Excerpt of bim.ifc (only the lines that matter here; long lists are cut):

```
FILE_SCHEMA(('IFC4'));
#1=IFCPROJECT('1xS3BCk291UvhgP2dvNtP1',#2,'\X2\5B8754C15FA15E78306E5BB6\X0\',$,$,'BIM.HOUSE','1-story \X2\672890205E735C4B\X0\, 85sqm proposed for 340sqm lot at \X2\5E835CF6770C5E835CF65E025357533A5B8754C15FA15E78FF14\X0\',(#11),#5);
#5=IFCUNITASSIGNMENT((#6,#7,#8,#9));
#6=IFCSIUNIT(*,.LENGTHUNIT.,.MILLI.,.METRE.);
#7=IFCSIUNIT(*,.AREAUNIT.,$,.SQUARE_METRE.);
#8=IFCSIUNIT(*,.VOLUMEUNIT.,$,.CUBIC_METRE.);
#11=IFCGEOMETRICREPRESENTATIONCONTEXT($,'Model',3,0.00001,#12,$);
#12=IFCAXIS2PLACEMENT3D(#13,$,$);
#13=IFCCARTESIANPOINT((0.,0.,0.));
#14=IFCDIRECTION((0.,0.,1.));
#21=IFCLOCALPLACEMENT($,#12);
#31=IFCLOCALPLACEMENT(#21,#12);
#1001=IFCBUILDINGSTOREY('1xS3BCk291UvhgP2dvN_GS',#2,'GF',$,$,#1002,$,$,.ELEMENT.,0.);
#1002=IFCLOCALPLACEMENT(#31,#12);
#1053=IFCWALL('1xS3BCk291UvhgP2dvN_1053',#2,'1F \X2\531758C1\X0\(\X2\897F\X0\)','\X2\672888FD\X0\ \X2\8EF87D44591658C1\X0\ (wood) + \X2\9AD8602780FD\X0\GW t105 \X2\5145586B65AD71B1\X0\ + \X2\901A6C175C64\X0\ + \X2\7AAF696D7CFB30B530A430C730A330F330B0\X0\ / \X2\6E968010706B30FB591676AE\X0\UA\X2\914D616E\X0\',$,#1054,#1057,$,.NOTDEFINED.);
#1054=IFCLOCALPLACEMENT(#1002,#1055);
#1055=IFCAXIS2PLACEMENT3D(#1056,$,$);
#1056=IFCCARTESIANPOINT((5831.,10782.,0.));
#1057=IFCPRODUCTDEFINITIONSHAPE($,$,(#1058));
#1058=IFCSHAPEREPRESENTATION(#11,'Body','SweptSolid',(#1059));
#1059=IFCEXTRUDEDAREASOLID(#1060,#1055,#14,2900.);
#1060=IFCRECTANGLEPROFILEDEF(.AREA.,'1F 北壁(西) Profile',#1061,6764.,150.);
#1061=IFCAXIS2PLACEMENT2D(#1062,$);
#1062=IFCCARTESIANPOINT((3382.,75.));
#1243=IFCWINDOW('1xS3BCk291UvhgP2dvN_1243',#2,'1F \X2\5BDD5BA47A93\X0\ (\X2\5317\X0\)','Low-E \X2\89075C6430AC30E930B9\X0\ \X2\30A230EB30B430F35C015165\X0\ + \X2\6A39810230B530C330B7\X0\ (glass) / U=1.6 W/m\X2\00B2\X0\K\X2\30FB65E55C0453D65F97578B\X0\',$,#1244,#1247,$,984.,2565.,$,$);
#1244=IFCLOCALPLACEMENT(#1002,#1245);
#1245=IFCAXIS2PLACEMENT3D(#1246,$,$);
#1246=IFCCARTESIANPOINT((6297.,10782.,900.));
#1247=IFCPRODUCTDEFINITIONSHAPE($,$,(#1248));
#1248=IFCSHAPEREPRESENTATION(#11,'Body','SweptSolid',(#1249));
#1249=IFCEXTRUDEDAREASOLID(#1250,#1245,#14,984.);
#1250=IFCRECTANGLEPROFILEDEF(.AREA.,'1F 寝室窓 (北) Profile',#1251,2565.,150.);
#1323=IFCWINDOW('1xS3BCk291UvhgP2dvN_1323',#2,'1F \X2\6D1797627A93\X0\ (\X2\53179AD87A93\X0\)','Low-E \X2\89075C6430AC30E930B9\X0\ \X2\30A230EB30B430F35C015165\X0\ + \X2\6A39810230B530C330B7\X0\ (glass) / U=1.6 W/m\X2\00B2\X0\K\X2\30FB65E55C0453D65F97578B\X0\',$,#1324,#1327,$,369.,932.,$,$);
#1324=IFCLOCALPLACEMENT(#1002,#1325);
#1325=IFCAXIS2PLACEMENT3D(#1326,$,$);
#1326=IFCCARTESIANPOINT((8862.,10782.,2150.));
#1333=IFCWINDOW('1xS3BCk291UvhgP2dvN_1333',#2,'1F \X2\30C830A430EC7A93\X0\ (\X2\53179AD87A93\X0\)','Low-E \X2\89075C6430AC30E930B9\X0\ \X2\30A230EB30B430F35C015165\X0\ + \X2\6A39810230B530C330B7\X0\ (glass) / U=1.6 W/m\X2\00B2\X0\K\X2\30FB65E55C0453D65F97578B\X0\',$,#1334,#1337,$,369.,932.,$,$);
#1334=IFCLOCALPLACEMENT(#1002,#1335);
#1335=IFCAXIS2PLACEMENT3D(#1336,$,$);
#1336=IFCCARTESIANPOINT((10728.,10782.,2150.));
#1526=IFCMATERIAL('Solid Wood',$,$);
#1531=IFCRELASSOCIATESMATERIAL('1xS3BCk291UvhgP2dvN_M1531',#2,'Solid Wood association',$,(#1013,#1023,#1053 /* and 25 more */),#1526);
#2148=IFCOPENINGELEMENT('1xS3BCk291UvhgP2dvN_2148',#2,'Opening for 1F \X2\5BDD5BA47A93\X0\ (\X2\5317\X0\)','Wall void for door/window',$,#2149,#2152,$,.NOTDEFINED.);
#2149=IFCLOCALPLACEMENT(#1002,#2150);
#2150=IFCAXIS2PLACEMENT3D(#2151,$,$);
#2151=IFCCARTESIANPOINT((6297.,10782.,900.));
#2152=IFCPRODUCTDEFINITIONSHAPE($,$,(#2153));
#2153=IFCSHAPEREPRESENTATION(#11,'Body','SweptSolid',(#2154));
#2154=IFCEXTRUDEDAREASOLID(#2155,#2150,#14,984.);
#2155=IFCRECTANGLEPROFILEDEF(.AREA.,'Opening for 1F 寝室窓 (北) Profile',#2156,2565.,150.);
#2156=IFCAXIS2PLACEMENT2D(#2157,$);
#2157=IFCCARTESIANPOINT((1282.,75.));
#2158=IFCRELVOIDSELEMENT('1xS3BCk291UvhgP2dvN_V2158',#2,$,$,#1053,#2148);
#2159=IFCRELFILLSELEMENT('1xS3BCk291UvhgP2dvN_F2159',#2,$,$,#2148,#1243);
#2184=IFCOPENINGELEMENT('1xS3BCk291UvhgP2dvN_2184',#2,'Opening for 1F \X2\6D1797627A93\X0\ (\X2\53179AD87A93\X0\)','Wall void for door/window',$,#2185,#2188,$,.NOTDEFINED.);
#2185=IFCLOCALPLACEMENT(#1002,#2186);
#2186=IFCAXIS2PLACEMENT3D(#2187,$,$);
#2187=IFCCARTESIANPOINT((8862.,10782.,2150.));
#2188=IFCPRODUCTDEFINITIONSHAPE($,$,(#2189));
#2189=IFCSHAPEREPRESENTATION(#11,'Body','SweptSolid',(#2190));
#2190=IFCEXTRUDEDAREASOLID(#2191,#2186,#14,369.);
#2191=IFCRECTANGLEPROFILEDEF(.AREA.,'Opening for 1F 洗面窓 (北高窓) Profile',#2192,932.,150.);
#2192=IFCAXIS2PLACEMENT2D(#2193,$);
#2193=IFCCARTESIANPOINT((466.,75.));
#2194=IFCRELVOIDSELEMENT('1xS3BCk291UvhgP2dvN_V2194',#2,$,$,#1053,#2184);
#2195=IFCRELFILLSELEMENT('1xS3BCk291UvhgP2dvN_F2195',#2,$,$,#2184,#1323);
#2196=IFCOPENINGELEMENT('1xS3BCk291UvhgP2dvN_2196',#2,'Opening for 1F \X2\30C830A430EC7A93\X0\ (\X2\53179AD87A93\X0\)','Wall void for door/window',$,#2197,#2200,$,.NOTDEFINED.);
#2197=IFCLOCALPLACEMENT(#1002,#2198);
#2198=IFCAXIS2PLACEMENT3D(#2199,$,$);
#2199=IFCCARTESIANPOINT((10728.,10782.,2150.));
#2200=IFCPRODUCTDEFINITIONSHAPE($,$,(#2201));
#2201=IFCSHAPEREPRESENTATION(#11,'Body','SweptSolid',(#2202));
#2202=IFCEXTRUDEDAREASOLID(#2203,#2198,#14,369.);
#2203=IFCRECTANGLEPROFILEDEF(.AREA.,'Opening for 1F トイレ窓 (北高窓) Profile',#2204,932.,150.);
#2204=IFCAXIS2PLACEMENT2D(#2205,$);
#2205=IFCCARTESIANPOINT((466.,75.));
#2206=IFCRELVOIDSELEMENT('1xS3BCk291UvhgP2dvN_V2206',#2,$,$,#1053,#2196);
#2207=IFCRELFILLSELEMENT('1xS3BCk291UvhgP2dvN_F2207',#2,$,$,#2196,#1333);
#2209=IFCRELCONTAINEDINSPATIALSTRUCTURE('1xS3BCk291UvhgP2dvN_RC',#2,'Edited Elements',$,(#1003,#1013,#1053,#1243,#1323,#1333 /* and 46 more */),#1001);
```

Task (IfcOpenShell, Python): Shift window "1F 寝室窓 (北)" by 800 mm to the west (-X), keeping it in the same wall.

```python
import ifcopenshell
import ifcopenshell.api.geometry
import ifcopenshell.util.placement

model = ifcopenshell.open("bim.ifc")

window = model.by_id(1243)
opening = window.FillsVoids[0].RelatingOpeningElement
wall = opening.VoidsElements[0].RelatingBuildingElement

wall_matrix = ifcopenshell.util.placement.get_local_placement(wall.ObjectPlacement)
shift = wall_matrix[:3, 0] * -800.0
before = ifcopenshell.util.placement.get_local_placement(window.ObjectPlacement)[:3, 3].copy()

# The window is not placed relative to its opening, so move both.
for product in (opening, window):
    matrix = ifcopenshell.util.placement.get_local_placement(product.ObjectPlacement)
    matrix[:3, 3] += shift
    ifcopenshell.api.geometry.edit_object_placement(model, product=product, matrix=matrix, is_si=False)

after = ifcopenshell.util.placement.get_local_placement(window.ObjectPlacement)[:3, 3]
print("window moved by", (after - before).round(3) + 0.0)

model.write("bim_v2.ifc")
```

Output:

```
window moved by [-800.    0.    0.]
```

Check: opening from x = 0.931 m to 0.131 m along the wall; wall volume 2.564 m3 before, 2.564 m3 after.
